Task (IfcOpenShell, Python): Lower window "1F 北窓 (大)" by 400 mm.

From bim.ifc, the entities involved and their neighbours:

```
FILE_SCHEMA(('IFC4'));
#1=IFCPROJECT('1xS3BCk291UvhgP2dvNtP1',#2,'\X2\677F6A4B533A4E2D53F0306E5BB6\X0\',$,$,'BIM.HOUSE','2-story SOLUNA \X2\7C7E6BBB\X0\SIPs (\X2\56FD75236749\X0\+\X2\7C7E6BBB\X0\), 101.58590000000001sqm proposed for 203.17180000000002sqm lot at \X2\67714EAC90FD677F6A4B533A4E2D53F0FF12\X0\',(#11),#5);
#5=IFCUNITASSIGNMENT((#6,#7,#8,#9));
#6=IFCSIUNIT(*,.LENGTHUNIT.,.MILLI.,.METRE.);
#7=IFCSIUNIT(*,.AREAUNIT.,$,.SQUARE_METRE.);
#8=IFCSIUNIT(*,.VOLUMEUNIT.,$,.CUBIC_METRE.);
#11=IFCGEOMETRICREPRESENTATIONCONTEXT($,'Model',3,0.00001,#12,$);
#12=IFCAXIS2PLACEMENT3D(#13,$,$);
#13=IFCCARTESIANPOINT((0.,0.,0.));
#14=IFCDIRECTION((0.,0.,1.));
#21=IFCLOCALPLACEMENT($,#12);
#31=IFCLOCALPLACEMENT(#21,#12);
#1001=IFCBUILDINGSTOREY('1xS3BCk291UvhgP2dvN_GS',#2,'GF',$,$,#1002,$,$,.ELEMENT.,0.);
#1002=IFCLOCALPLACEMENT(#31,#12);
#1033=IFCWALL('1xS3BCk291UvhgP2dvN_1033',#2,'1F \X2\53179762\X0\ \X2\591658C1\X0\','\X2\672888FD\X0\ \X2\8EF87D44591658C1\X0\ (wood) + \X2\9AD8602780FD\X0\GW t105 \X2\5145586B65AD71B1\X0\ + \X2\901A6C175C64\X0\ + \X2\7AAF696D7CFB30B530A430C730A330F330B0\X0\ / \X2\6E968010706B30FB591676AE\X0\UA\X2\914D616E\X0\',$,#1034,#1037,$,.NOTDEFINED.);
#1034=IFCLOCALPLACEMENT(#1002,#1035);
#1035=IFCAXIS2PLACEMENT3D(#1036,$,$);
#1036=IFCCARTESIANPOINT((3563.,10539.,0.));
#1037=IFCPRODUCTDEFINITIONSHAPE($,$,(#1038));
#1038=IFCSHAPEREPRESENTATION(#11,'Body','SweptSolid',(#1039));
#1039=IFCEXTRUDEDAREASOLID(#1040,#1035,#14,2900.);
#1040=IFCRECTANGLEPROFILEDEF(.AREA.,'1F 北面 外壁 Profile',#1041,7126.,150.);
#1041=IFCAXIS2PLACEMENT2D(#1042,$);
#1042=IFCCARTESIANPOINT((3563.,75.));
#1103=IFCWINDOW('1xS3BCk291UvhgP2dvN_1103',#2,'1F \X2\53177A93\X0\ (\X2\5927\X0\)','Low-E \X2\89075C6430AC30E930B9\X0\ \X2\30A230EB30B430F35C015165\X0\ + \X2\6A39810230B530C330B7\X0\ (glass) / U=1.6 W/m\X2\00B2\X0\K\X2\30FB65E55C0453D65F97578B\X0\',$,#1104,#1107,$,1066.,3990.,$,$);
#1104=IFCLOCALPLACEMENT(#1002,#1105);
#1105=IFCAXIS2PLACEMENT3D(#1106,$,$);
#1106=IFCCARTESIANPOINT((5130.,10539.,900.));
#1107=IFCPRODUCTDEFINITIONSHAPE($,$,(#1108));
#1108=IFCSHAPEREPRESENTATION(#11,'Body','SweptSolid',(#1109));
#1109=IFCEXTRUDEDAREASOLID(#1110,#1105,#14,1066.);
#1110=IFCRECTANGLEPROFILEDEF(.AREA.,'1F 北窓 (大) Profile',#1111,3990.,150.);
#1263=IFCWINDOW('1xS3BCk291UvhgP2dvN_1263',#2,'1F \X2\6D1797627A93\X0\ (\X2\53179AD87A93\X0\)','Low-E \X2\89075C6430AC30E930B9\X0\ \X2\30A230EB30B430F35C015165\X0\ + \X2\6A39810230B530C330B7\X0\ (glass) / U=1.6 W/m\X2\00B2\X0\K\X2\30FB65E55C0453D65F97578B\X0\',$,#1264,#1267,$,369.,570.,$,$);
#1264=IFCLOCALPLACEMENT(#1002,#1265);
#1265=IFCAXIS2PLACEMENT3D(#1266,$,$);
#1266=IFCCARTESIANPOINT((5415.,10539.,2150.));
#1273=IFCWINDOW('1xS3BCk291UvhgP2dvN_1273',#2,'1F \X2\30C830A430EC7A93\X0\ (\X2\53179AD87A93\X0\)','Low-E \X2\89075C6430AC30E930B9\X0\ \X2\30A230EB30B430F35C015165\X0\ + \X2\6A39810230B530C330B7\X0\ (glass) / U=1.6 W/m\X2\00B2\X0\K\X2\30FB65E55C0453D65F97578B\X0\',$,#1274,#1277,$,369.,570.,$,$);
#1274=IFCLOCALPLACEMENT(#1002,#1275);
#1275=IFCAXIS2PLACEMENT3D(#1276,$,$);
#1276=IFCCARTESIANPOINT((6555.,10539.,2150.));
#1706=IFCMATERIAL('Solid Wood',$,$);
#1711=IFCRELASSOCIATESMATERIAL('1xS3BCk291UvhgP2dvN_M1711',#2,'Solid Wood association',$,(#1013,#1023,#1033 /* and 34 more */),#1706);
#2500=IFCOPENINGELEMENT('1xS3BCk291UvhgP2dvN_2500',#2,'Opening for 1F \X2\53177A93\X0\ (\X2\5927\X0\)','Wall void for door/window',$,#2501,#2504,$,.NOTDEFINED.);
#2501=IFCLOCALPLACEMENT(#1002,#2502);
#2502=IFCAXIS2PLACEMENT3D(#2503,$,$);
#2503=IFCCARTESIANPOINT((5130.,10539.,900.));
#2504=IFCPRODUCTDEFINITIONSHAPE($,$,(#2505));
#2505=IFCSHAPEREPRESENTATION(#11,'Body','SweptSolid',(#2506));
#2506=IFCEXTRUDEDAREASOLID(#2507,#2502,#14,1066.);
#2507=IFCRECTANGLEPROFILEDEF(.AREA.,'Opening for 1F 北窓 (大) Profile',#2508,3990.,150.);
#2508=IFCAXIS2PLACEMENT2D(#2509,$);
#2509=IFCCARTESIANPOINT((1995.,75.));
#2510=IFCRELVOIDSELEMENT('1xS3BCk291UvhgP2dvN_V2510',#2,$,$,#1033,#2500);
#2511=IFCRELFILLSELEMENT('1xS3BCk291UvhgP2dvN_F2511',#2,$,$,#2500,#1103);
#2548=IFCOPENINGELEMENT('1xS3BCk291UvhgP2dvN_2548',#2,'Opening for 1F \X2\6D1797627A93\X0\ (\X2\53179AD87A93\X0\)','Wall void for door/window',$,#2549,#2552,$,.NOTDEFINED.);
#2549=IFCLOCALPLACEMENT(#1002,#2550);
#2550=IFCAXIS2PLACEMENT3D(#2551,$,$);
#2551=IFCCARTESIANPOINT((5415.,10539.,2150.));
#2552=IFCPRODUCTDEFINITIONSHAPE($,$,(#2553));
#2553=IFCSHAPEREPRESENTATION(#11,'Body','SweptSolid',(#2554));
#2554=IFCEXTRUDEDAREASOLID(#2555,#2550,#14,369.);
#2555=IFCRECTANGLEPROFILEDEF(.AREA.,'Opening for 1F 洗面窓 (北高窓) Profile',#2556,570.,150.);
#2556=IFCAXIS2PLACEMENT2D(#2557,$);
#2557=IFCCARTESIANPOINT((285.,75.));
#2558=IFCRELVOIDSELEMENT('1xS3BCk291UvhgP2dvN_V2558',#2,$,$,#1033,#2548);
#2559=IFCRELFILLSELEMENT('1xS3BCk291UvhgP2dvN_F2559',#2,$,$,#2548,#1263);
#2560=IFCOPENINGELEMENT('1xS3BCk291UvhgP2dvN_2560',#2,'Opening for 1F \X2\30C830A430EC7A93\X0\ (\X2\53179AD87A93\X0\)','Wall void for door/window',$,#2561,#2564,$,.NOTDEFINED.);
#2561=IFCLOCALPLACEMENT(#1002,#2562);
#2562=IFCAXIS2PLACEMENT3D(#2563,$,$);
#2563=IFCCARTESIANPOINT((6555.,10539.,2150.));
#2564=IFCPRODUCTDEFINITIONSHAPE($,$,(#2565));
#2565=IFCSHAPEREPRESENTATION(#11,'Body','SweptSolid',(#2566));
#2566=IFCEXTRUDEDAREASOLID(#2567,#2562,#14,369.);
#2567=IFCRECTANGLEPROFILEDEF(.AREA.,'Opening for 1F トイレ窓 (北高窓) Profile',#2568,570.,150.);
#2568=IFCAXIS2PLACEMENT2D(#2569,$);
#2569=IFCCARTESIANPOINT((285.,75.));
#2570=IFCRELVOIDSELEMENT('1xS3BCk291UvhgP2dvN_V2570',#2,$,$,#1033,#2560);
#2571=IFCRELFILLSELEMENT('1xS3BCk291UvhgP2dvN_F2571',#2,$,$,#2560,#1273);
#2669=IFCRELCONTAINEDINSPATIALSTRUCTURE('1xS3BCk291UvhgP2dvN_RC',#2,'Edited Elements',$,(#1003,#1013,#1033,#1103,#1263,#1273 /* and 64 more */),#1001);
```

```python
import numpy as np
import ifcopenshell
import ifcopenshell.api.geometry
import ifcopenshell.util.placement
import ifcopenshell.util.unit

model = ifcopenshell.open("bim.ifc")
unit_scale = ifcopenshell.util.unit.calculate_unit_scale(model)

window = model.by_guid("1xS3BCk291UvhgP2dvN_1103")
opening = window.FillsVoids[0].RelatingOpeningElement
dz = -400.0

shift = np.array([0.0, 0.0, dz])
# The window is not placed relative to its opening, so move both.
for product in (opening, window):
    matrix = ifcopenshell.util.placement.get_local_placement(product.ObjectPlacement)
    matrix[:3, 3] += shift
    ifcopenshell.api.geometry.edit_object_placement(model, product=product, matrix=matrix, is_si=False)

print(f"moved by {dz * unit_scale:+.3f} m")

model.write("bim_updated.ifc")
```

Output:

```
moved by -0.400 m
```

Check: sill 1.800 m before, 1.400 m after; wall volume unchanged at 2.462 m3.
